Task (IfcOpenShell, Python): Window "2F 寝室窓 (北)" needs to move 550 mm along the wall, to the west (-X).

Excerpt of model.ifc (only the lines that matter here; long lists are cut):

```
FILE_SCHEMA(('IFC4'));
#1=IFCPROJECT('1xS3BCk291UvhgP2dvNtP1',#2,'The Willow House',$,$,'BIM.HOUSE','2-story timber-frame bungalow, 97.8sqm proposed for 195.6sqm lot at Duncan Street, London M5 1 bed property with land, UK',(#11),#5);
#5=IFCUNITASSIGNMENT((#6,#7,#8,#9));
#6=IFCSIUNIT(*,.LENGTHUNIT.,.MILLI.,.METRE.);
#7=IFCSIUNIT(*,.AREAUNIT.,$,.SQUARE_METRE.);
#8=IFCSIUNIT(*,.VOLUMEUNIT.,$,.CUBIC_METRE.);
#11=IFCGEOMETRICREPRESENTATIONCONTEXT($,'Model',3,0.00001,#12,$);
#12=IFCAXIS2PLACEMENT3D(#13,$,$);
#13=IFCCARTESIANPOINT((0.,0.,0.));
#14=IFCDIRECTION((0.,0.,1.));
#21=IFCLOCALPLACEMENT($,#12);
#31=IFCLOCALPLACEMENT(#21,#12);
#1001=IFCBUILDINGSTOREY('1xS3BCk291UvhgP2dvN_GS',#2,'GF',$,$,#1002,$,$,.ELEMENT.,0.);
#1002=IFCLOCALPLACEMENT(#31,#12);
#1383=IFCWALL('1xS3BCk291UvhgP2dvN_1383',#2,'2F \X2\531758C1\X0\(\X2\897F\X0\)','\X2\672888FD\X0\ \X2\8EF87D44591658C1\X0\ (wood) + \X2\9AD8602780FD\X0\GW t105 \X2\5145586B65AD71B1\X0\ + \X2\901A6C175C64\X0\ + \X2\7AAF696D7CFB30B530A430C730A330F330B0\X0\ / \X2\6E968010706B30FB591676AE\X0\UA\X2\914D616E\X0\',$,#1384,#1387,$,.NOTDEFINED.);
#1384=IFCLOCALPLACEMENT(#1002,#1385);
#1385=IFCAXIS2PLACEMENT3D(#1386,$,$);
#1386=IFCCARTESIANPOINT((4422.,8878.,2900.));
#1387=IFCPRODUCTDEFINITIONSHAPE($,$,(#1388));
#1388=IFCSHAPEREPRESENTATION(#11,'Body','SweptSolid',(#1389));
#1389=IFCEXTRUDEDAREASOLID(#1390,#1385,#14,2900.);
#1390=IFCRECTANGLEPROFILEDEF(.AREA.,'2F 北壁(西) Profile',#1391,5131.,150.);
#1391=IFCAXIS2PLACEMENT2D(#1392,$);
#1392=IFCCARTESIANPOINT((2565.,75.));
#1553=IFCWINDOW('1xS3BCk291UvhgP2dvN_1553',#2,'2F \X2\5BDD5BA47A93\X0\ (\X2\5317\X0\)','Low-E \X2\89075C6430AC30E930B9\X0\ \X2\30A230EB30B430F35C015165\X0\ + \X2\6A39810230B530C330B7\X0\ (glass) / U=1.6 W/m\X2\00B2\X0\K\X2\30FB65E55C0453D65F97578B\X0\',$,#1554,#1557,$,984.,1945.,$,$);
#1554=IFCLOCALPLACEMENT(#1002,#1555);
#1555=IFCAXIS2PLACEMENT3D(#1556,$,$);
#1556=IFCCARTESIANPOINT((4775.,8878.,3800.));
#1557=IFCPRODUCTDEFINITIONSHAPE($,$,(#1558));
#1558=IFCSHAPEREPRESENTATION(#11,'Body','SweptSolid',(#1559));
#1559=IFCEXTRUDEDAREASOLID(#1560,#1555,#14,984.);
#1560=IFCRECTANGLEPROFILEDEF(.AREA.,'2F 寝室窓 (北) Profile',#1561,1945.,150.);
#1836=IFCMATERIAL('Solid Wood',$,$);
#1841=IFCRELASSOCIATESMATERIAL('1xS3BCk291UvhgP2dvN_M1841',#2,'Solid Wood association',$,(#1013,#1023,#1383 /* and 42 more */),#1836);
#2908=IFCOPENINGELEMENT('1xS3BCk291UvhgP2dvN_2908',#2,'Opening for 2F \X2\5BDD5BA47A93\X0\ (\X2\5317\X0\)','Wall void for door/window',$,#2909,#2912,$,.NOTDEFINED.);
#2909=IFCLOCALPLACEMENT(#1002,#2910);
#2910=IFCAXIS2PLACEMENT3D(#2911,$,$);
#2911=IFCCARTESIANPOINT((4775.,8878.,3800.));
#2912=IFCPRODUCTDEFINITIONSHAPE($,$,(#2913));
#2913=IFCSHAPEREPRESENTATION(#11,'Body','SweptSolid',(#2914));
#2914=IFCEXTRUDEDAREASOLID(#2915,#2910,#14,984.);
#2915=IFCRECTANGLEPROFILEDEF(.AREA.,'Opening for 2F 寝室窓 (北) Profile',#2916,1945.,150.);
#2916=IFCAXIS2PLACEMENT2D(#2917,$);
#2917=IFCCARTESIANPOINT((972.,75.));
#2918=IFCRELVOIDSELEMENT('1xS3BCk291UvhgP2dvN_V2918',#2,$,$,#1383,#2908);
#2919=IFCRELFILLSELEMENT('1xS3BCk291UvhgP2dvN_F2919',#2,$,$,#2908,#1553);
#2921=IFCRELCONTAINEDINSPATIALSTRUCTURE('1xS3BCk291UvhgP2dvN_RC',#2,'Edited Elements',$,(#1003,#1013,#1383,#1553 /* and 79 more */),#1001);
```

```python
import ifcopenshell
import ifcopenshell.api.geometry
import ifcopenshell.util.placement
import ifcopenshell.util.unit

model = ifcopenshell.open("model.ifc")
unit_scale = ifcopenshell.util.unit.calculate_unit_scale(model)

window = model.by_guid("1xS3BCk291UvhgP2dvN_1553")
opening = window.FillsVoids[0].RelatingOpeningElement
wall = opening.VoidsElements[0].RelatingBuildingElement

wall_matrix = ifcopenshell.util.placement.get_local_placement(wall.ObjectPlacement)
shift = wall_matrix[:3, 0] * -0.55 / unit_scale
before = ifcopenshell.util.placement.get_local_placement(window.ObjectPlacement)[:3, 3].copy()

# The window is not placed relative to its opening, so move both.
for product in (opening, window):
    matrix = ifcopenshell.util.placement.get_local_placement(product.ObjectPlacement)
    matrix[:3, 3] += shift
    ifcopenshell.api.geometry.edit_object_placement(model, product=product, matrix=matrix, is_si=False)

after = ifcopenshell.util.placement.get_local_placement(window.ObjectPlacement)[:3, 3]
print("window moved by", (after - before).round(3) + 0.0)

model.write("model_v2.ifc")
```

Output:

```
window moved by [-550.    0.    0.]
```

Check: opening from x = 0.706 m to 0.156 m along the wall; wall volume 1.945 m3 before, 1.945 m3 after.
